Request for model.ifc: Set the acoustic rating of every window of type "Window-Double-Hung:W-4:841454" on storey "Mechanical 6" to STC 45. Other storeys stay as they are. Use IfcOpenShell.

First a look at what the model holds.

```python
import ifcopenshell
import ifcopenshell.util.element

model = ifcopenshell.open("model.ifc")
print(model.schema)
storey = next(s for s in model.by_type("IfcBuildingStorey") if s.Name == "Mechanical 6")
windows = [e for e in ifcopenshell.util.element.get_decomposition(storey) if e.is_a("IfcWindow")]
seen = {}
for e in windows:
    element_type = ifcopenshell.util.element.get_type(e)
    key = (element_type.Name if element_type != e and element_type else None, ifcopenshell.util.element.get_pset(e, "Pset_WindowCommon", "AcousticRating"))
    seen[key] = seen.get(key, 0) + 1
for (name, value), count in sorted(seen.items(), key=str):
    print(count, "x", name, "|", value)
```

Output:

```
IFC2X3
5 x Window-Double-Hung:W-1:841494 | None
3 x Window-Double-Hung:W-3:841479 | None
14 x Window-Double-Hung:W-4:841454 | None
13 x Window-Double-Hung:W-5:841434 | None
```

```python
import ifcopenshell
import ifcopenshell.api.pset
import ifcopenshell.util.element

model = ifcopenshell.open("model.ifc")

storey = next(s for s in model.by_type("IfcBuildingStorey") if s.Name == "Mechanical 6")
windows = [e for e in ifcopenshell.util.element.get_decomposition(storey) if e.is_a("IfcWindow")]

count = 0
for e in windows:
    element_type = ifcopenshell.util.element.get_type(e)
    if element_type in (None, e) or element_type.Name != "Window-Double-Hung:W-4:841454":
        continue
    # add_pset returns the element's existing set when there is one.
    pset = ifcopenshell.api.pset.add_pset(model, product=e, name="Pset_WindowCommon")
    ifcopenshell.api.pset.edit_pset(model, pset=pset, properties={"AcousticRating": "STC 45"})
    count += 1

print(count, "windows updated")

model.write("model_v2.ifc")
```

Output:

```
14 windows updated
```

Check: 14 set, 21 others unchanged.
